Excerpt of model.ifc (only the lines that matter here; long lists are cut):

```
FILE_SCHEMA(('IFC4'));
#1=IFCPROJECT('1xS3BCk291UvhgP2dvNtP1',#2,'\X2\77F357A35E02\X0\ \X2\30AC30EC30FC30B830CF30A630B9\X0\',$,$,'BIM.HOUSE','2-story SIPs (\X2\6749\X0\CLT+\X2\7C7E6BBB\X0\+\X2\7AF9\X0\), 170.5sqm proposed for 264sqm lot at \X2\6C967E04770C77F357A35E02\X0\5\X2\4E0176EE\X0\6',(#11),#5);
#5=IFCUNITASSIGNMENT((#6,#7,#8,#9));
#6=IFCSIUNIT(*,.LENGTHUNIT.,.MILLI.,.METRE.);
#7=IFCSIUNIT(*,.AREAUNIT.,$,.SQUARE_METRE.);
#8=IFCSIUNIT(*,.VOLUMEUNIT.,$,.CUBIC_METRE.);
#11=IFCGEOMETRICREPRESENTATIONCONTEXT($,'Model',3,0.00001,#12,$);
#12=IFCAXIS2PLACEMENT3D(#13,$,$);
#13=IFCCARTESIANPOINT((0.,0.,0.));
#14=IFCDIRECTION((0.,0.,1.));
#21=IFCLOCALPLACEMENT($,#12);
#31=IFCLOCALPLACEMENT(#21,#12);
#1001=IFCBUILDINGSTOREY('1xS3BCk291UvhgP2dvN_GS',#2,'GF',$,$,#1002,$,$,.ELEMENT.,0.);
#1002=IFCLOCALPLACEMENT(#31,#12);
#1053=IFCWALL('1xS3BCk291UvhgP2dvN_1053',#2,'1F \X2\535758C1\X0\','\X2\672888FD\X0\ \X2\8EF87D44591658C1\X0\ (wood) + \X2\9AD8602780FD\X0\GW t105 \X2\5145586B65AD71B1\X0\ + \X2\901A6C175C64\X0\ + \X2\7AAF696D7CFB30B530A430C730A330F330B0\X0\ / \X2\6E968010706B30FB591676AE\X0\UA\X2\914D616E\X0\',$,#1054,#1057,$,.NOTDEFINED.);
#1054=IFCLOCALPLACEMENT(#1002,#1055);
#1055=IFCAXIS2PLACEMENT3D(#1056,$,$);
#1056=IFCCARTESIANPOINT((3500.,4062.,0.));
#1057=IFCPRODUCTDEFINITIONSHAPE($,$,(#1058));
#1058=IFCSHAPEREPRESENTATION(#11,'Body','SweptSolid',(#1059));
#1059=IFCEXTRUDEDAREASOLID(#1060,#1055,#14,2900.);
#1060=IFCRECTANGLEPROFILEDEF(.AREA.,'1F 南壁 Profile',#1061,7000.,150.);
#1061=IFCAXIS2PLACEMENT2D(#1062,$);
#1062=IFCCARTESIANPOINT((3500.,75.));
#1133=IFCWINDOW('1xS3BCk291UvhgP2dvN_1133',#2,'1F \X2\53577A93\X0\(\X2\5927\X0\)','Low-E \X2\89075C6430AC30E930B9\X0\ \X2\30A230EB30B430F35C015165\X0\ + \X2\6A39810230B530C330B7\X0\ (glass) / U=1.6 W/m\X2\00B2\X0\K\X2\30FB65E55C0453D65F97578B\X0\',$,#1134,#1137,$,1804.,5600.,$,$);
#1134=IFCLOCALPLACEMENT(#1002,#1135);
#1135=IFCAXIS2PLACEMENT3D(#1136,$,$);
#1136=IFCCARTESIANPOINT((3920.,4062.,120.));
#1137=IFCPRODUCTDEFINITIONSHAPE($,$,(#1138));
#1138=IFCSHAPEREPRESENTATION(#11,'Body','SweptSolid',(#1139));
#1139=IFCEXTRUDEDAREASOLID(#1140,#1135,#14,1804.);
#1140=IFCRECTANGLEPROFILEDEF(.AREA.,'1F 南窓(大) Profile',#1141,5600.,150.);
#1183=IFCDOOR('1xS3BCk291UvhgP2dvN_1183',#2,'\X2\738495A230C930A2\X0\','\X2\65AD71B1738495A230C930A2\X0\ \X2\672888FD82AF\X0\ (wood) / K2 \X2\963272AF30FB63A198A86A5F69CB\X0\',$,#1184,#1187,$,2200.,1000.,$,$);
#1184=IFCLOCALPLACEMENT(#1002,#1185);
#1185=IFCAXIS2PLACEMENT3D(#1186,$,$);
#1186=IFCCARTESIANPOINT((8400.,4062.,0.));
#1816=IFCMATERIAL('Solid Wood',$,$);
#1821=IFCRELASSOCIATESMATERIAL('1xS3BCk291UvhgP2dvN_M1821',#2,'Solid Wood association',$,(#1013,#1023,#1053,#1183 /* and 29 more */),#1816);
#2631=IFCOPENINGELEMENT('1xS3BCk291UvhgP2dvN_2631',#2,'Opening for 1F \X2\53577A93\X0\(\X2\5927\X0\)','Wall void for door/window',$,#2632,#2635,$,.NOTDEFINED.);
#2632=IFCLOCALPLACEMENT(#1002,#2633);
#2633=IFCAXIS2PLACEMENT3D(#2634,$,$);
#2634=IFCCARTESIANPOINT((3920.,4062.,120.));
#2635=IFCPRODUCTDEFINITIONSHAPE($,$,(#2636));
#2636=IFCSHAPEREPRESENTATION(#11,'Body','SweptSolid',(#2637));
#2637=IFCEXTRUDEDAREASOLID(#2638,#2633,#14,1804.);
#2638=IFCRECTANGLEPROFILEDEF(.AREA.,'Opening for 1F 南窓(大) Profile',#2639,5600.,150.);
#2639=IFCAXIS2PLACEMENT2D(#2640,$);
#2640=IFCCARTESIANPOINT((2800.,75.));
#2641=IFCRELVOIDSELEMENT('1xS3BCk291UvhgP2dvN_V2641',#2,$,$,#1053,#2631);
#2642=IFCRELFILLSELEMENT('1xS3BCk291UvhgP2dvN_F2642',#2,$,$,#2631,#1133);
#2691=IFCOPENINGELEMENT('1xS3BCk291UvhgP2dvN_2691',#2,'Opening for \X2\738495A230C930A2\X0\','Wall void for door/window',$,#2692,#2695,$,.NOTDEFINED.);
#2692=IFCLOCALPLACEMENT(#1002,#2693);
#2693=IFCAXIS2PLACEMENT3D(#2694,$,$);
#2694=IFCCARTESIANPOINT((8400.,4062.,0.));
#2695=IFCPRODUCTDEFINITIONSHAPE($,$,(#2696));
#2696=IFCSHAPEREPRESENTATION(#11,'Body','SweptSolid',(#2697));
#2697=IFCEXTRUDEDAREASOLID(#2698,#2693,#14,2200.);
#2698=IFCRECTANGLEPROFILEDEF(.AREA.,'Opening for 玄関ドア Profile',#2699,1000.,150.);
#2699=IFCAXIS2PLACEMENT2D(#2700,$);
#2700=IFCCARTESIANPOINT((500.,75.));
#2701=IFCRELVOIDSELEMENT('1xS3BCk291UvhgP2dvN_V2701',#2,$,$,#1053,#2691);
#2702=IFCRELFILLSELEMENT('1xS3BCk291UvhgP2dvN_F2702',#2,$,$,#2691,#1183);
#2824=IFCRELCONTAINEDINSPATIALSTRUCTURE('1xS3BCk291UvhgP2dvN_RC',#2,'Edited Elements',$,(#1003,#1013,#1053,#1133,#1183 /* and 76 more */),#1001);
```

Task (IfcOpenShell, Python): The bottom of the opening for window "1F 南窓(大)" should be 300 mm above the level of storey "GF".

```python
import numpy as np
import ifcopenshell
import ifcopenshell.api.geometry
import ifcopenshell.geom
import ifcopenshell.util.element
import ifcopenshell.util.placement
import ifcopenshell.util.shape
import ifcopenshell.util.unit

model = ifcopenshell.open("model.ifc")
unit_scale = ifcopenshell.util.unit.calculate_unit_scale(model)

window = model.by_guid("1xS3BCk291UvhgP2dvN_1133")
opening = window.FillsVoids[0].RelatingOpeningElement
storey = ifcopenshell.util.element.get_container(window, ifc_class="IfcBuildingStorey")
level = ifcopenshell.util.placement.get_local_placement(storey.ObjectPlacement)[2, 3]

# The opening's origin need not be at the sill, so measure its lowest point.
shape = ifcopenshell.geom.create_shape(ifcopenshell.geom.settings(), opening)
bottom = ifcopenshell.util.shape.get_shape_bottom_elevation(shape, shape.geometry) / unit_scale
dz = level + 0.3 / unit_scale - bottom

shift = np.array([0.0, 0.0, dz])
# The window is not placed relative to its opening, so move both.
for product in (opening, window):
    matrix = ifcopenshell.util.placement.get_local_placement(product.ObjectPlacement)
    matrix[:3, 3] += shift
    ifcopenshell.api.geometry.edit_object_placement(model, product=product, matrix=matrix, is_si=False)

print(f"moved by {dz * unit_scale:+.3f} m")

model.write("model_rev.ifc")
```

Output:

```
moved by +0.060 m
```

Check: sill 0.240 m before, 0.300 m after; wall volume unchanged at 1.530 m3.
